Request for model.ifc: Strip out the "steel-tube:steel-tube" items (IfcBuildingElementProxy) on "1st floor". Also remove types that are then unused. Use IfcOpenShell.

First a look at what the model holds.

```python
import ifcopenshell
import ifcopenshell.util.element

model = ifcopenshell.open("model.ifc")
print(model.schema)
storey = next(s for s in model.by_type("IfcBuildingStorey") if s.Name == "1st floor")
proxies = [e for e in ifcopenshell.util.element.get_decomposition(storey) if e.is_a("IfcBuildingElementProxy")]
seen = {}
for e in proxies:
    element_type = ifcopenshell.util.element.get_type(e)
    name = element_type.Name if element_type not in (None, e) else None
    seen[name] = seen.get(name, 0) + 1
for name, count in sorted(seen.items(), key=str):
    print(count, "x", name)
```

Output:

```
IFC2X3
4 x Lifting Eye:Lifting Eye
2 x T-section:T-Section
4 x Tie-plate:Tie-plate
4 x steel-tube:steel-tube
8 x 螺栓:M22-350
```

```python
import ifcopenshell
import ifcopenshell.api.root
import ifcopenshell.util.element

model = ifcopenshell.open("model.ifc")

storey = next(s for s in model.by_type("IfcBuildingStorey") if s.Name == "1st floor")
proxies = [e for e in ifcopenshell.util.element.get_decomposition(storey) if e.is_a("IfcBuildingElementProxy")]
targets = [e for e in proxies if (t := ifcopenshell.util.element.get_type(e)) not in (None, e) and t.Name == "steel-tube:steel-tube"]
types = {ifcopenshell.util.element.get_type(e) for e in targets} - {None, *targets}

for e in targets:
    ifcopenshell.api.root.remove_product(model, product=e)
print(len(targets), "removed")

unused = [t for t in types if not ifcopenshell.util.element.get_types(t)]
for t in unused:
    ifcopenshell.api.root.remove_product(model, product=t)
print(len(unused), "unused types removed")

model.write("model_edited.ifc")
```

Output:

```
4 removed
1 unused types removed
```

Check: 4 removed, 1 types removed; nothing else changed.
